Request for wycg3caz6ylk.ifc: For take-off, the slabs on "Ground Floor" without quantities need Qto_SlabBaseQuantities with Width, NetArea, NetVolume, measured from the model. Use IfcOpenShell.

First a look at what the model holds.

```python
import ifcopenshell
import ifcopenshell.util.element
import ifcopenshell.util.unit

model = ifcopenshell.open("wycg3caz6ylk.ifc")
print(model.schema)
for unit_type in ("LENGTHUNIT", "AREAUNIT", "VOLUMEUNIT"):
    print(unit_type, ifcopenshell.util.unit.calculate_unit_scale(model, unit_type))
storey = next(s for s in model.by_type("IfcBuildingStorey") if s.Name == "Ground Floor")
slabs = [e for e in ifcopenshell.util.element.get_decomposition(storey) if e.is_a("IfcSlab")]
for e in sorted(slabs, key=lambda e: e.id()):
    print(e.id(), e.is_a(), e.Name, list(ifcopenshell.util.element.get_psets(e, qtos_only=True)), sep=" | ")
```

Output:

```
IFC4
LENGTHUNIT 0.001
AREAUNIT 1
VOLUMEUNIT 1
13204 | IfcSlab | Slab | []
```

```python
import ifcopenshell
import ifcopenshell.api.pset
import ifcopenshell.geom
import ifcopenshell.util.element
import ifcopenshell.util.shape
import ifcopenshell.util.unit

model = ifcopenshell.open("wycg3caz6ylk.ifc")
unit_scale = ifcopenshell.util.unit.calculate_unit_scale(model)
area_scale = ifcopenshell.util.unit.calculate_unit_scale(model, "AREAUNIT")
volume_scale = ifcopenshell.util.unit.calculate_unit_scale(model, "VOLUMEUNIT")
settings = ifcopenshell.geom.settings()

storey = next(s for s in model.by_type("IfcBuildingStorey") if s.Name == "Ground Floor")
slabs = [e for e in ifcopenshell.util.element.get_decomposition(storey) if e.is_a("IfcSlab")]

for e in sorted(slabs, key=lambda e: e.id()):
    if ifcopenshell.util.element.get_psets(e, qtos_only=True, should_inherit=False):
        continue
    # Geometry comes back in metres, in the element's own axes.
    shape = ifcopenshell.geom.create_shape(settings, e)
    values = {
        "Width": ifcopenshell.util.shape.get_z(shape.geometry) / unit_scale,
        "NetArea": ifcopenshell.util.shape.get_footprint_area(shape.geometry) / area_scale,
        "NetVolume": ifcopenshell.util.shape.get_volume(shape.geometry) / volume_scale,
    }
    qto = ifcopenshell.api.pset.add_qto(model, product=e, name="Qto_SlabBaseQuantities")
    ifcopenshell.api.pset.edit_qto(model, qto=qto, properties=values)
    print(e.id(), {k: round(v, 3) for k, v in values.items()})

model.write("wycg3caz6ylk_updated.ifc")
```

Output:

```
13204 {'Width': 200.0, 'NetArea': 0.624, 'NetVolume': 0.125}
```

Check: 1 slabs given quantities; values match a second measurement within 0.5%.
